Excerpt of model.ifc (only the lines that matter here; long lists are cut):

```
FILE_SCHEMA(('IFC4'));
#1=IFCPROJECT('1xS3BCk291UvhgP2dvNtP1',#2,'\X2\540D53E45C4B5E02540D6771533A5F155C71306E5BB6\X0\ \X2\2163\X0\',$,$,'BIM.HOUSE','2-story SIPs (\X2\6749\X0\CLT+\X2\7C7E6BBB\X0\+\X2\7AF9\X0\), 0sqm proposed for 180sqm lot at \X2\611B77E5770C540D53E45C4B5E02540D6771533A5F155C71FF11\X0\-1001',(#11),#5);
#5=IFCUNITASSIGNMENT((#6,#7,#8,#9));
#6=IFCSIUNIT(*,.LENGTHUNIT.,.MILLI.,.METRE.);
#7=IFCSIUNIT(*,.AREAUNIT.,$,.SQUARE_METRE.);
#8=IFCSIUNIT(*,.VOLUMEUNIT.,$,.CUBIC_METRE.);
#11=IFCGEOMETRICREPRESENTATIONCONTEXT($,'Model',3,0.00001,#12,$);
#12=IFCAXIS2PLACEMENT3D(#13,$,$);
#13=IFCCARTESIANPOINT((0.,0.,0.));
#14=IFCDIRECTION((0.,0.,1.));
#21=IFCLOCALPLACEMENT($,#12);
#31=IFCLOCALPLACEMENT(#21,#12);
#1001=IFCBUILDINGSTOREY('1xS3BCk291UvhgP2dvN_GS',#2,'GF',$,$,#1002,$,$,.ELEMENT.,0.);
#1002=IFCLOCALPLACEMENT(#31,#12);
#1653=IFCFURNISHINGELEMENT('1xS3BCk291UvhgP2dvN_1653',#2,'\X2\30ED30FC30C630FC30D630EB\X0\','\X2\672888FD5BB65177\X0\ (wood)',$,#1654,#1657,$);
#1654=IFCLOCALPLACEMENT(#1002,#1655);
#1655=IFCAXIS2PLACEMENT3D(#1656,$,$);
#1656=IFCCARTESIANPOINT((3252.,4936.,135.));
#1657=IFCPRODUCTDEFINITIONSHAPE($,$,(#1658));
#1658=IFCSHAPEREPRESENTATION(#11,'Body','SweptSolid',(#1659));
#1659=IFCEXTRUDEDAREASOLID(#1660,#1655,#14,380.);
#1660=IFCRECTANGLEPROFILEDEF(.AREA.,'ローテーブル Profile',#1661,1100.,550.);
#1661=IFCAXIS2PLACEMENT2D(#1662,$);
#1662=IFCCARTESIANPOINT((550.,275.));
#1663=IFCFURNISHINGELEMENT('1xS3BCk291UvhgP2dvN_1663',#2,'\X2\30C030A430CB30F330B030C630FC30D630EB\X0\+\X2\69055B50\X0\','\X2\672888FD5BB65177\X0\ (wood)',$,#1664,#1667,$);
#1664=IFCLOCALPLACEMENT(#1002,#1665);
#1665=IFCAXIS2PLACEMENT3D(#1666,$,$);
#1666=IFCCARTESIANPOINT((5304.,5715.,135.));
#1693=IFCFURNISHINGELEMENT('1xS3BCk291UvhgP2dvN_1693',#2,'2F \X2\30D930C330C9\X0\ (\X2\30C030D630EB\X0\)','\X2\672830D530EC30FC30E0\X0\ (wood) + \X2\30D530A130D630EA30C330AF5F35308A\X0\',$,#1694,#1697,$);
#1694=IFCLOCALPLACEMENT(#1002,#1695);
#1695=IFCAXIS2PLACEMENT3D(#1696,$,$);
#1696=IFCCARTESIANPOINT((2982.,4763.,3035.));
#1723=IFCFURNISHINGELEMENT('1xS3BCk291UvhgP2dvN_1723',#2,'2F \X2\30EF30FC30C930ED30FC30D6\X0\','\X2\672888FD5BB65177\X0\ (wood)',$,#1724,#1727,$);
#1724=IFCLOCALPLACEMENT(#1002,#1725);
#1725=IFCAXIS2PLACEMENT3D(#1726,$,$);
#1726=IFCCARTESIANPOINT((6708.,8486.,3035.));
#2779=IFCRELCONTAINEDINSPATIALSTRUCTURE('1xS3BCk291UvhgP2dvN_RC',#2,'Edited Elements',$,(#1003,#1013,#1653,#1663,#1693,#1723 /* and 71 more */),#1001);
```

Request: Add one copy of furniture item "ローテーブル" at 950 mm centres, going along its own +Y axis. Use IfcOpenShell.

```python
import ifcopenshell
import ifcopenshell.api.geometry
import ifcopenshell.api.root
import ifcopenshell.util.element
import ifcopenshell.util.placement

model = ifcopenshell.open("model.ifc")


def reuse_history(source, copy):
    """copy_class also copies each property set's owner history, people and application; keep the originals."""
    for rel in copy.IsDefinedBy:
        if rel.is_a("IfcRelDefinesByProperties") and (history := rel.RelatingPropertyDefinition.OwnerHistory):
            rel.RelatingPropertyDefinition.OwnerHistory = source.OwnerHistory
            ifcopenshell.util.element.remove_deep2(model, history)


source = model.by_guid("1xS3BCk291UvhgP2dvN_1653")
base = ifcopenshell.util.placement.get_local_placement(source.ObjectPlacement)
step = base[:3, 1] * 950.0

for i in range(1, 2):
    copy = ifcopenshell.api.root.copy_class(model, product=source)
    copy.Representation = ifcopenshell.util.element.copy_deep(
        model, source.Representation, exclude=["IfcGeometricRepresentationContext", "IfcRepresentationMap"]
    )
    reuse_history(source, copy)
    matrix = base.copy()
    matrix[:3, 3] += i * step
    print("added at", matrix[:3, 3].round(3) + 0.0)
    ifcopenshell.api.geometry.edit_object_placement(model, product=copy, matrix=matrix, is_si=False)

model.write("model-out.ifc")
```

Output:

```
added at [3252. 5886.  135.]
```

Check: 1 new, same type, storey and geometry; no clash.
